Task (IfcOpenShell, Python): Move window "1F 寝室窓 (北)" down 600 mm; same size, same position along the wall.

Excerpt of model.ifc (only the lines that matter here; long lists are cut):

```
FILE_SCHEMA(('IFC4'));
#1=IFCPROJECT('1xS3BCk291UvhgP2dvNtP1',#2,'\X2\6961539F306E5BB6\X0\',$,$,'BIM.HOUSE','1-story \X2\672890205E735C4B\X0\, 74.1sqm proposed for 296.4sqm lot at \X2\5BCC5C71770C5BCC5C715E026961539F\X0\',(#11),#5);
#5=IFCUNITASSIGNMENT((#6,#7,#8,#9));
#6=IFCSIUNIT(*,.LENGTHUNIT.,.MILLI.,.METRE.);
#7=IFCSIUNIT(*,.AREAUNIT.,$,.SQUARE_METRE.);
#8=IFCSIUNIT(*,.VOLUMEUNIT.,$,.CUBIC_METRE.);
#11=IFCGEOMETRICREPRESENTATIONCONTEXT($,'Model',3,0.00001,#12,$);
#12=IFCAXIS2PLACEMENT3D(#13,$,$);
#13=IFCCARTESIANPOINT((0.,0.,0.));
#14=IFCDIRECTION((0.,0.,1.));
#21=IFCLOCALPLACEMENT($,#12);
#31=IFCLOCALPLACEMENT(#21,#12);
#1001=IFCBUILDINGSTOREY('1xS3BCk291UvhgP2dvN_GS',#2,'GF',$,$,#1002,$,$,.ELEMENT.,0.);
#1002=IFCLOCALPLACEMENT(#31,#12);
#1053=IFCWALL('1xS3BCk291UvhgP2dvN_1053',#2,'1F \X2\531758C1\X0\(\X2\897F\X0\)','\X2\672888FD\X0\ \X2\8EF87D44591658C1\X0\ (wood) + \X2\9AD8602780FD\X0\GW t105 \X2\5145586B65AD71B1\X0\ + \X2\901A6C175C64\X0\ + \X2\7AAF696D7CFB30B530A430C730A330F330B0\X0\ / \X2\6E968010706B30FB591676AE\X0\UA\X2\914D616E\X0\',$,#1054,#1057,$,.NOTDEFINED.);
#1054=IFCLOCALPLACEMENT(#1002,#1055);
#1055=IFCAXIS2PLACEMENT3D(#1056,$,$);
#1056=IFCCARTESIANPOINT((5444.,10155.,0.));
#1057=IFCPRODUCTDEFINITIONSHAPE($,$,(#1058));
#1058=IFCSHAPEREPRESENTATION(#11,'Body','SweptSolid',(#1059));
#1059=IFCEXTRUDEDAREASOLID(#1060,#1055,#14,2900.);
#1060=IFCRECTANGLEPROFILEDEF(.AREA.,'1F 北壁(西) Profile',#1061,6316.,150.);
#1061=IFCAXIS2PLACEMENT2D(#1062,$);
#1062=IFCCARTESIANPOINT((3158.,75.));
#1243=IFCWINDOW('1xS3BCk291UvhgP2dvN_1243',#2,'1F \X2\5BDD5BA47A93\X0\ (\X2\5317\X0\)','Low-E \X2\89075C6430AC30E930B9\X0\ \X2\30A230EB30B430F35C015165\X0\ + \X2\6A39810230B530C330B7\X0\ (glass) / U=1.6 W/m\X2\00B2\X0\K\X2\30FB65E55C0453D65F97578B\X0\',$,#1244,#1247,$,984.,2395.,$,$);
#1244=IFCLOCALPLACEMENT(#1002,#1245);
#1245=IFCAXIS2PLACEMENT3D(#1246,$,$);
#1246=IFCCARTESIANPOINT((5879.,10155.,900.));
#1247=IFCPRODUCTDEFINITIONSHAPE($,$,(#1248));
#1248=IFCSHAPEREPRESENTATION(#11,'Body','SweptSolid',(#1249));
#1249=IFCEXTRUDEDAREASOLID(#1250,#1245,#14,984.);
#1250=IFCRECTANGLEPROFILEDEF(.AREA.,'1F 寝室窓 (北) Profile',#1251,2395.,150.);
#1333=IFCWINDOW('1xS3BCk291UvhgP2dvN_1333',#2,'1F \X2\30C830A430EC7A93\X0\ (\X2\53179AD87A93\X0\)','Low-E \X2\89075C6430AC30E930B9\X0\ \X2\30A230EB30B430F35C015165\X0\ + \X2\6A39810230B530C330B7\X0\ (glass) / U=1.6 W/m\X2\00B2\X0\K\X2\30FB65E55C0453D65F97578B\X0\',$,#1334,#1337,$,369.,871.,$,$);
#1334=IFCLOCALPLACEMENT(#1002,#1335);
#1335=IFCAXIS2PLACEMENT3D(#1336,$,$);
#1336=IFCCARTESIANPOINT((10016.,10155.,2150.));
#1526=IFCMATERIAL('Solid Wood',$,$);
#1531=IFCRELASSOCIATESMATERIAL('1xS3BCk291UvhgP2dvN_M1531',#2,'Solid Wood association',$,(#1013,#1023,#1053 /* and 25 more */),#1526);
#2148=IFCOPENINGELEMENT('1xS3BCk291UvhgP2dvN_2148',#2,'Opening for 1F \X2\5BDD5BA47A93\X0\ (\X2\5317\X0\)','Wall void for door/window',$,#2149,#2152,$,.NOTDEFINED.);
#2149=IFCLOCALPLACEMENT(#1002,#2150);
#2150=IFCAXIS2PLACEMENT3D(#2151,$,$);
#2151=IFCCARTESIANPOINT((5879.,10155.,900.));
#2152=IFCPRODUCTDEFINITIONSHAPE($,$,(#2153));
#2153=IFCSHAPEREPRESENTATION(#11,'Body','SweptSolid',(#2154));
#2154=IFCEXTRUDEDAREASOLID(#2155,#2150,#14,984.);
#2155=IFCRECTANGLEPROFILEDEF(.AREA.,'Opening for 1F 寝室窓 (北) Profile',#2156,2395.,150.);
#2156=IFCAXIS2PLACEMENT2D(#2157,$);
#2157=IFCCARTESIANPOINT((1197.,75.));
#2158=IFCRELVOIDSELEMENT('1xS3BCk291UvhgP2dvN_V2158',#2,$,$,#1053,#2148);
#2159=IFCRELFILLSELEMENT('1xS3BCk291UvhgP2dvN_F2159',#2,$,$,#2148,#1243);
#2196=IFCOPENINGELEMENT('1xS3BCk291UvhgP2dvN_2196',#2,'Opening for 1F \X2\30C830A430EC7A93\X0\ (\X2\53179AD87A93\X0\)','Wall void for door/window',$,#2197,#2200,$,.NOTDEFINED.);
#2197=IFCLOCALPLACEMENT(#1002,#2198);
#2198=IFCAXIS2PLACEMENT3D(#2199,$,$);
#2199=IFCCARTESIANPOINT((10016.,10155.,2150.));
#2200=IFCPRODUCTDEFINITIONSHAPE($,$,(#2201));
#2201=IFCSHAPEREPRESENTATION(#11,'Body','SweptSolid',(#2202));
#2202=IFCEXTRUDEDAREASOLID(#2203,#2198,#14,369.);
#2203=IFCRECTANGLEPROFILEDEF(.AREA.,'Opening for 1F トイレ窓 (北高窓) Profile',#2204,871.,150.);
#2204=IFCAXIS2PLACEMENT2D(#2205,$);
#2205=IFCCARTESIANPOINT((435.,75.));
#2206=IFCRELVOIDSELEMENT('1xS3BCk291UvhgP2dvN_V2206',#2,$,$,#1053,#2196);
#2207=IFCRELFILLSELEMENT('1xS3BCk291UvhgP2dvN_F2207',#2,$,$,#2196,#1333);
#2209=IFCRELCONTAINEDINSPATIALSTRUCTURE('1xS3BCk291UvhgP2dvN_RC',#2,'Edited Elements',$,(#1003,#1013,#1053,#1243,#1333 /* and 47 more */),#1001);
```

```python
import numpy as np
import ifcopenshell
import ifcopenshell.api.geometry
import ifcopenshell.util.placement
import ifcopenshell.util.unit

model = ifcopenshell.open("model.ifc")
unit_scale = ifcopenshell.util.unit.calculate_unit_scale(model)

window = model.by_id(1243)
opening = window.FillsVoids[0].RelatingOpeningElement
dz = -0.6 / unit_scale

shift = np.array([0.0, 0.0, dz])
# The window is not placed relative to its opening, so move both.
for product in (opening, window):
    matrix = ifcopenshell.util.placement.get_local_placement(product.ObjectPlacement)
    matrix[:3, 3] += shift
    ifcopenshell.api.geometry.edit_object_placement(model, product=product, matrix=matrix, is_si=False)

print(f"moved by {dz * unit_scale:+.3f} m")

model.write("model_edited.ifc")
```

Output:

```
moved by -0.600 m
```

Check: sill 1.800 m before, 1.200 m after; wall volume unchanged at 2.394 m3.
